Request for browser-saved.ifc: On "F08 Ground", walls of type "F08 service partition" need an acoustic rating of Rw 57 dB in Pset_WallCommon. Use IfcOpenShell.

First a look at what the model holds.

```python
import ifcopenshell
import ifcopenshell.util.element

model = ifcopenshell.open("browser-saved.ifc")
print(model.schema)
storey = next(s for s in model.by_type("IfcBuildingStorey") if s.Name == "F08 Ground")
walls = [e for e in ifcopenshell.util.element.get_decomposition(storey) if e.is_a("IfcWall")]
seen = {}
for e in walls:
    element_type = ifcopenshell.util.element.get_type(e)
    key = (element_type.Name if element_type != e and element_type else None, ifcopenshell.util.element.get_pset(e, "Pset_WallCommon", "AcousticRating"))
    seen[key] = seen.get(key, 0) + 1
for (name, value), count in sorted(seen.items(), key=str):
    print(count, "x", name, "|", value)
```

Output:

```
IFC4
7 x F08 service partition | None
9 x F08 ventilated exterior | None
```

```python
import ifcopenshell
import ifcopenshell.api.pset
import ifcopenshell.util.element

model = ifcopenshell.open("browser-saved.ifc")

storey = next(s for s in model.by_type("IfcBuildingStorey") if s.Name == "F08 Ground")
walls = [e for e in ifcopenshell.util.element.get_decomposition(storey) if e.is_a("IfcWall")]

count = 0
for e in walls:
    element_type = ifcopenshell.util.element.get_type(e)
    if element_type in (None, e) or element_type.Name != "F08 service partition":
        continue
    # add_pset returns the element's existing set when there is one.
    pset = ifcopenshell.api.pset.add_pset(model, product=e, name="Pset_WallCommon")
    ifcopenshell.api.pset.edit_pset(model, pset=pset, properties={"AcousticRating": "Rw 57 dB"})
    count += 1

print(count, "walls updated")

model.write("browser-saved_edited.ifc")
```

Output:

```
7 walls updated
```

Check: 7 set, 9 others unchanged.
